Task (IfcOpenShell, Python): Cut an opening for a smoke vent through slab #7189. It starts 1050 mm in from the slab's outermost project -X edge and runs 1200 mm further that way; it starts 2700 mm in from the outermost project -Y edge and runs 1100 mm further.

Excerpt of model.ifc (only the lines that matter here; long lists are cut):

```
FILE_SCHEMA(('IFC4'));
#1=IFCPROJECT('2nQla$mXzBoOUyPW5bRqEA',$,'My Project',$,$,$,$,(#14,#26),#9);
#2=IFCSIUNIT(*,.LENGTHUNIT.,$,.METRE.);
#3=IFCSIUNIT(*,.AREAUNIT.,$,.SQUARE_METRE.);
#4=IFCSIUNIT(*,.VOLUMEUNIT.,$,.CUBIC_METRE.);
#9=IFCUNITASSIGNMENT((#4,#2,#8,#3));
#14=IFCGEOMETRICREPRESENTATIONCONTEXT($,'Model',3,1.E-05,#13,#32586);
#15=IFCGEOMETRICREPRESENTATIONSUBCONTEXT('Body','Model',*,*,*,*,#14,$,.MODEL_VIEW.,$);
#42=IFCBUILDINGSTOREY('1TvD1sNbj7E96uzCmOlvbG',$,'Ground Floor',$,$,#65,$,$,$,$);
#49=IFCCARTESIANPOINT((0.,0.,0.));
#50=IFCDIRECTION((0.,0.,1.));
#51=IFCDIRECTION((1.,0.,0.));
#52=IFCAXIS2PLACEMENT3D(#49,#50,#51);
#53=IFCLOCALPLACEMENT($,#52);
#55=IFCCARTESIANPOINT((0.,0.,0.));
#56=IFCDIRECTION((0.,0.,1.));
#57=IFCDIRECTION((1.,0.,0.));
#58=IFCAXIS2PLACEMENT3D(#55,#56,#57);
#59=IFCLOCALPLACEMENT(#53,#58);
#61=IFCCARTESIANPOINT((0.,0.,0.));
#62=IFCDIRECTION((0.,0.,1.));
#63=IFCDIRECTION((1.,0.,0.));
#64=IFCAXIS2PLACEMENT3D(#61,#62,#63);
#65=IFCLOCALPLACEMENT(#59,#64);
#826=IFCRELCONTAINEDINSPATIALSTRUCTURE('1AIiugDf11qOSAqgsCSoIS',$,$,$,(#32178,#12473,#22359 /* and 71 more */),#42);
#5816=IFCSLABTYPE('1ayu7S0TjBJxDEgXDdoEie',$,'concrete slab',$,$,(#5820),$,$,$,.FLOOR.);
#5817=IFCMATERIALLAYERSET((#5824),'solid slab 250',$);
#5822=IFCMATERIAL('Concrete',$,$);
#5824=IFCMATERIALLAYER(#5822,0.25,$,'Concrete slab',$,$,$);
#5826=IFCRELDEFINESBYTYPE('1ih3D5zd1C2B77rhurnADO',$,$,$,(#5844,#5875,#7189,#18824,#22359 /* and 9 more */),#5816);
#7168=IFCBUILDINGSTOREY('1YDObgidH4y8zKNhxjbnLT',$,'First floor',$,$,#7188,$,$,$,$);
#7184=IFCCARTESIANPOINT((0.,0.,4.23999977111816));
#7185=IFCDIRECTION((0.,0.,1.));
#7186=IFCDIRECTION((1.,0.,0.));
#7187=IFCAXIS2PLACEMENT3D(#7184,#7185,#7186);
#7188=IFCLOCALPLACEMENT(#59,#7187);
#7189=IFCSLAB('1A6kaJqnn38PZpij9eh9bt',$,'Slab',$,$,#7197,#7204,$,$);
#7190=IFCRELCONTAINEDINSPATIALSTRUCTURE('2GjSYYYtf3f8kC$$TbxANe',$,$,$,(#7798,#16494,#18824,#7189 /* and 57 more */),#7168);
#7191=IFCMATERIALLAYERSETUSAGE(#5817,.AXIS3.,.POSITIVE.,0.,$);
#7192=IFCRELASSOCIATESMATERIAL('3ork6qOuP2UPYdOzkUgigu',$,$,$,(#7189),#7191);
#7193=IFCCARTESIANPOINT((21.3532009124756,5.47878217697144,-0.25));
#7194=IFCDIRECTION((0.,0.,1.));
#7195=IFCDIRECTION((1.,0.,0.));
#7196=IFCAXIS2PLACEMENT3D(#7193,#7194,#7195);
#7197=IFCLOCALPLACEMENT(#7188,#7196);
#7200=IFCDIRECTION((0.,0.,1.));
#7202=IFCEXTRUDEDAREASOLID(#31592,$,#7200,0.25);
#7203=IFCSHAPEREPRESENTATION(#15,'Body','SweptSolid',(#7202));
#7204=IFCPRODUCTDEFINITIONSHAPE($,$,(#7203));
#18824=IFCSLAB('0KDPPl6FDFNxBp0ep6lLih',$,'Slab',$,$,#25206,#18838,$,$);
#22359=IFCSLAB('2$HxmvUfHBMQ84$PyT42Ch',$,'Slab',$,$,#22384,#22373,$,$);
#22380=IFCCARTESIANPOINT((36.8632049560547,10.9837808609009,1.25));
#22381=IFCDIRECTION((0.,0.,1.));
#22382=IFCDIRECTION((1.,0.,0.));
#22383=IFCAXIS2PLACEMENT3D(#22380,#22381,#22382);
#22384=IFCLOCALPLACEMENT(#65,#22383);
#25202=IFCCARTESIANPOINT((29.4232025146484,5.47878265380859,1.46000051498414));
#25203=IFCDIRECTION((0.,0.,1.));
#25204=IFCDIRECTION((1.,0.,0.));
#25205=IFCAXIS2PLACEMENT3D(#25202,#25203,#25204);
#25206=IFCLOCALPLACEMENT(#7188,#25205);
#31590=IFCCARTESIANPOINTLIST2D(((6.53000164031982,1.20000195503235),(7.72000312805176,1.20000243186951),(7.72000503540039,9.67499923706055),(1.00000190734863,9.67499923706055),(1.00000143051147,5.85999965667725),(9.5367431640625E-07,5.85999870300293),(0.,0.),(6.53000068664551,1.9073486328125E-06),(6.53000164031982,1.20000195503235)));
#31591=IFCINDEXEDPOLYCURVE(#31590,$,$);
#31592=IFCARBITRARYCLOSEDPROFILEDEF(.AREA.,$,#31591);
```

```python
import numpy as np
import ifcopenshell
import ifcopenshell.api.feature
import ifcopenshell.api.geometry
import ifcopenshell.api.root
import ifcopenshell.geom
import ifcopenshell.util.placement
import ifcopenshell.util.representation
import ifcopenshell.util.shape
import ifcopenshell.util.unit

model = ifcopenshell.open("model.ifc")
unit_scale = ifcopenshell.util.unit.calculate_unit_scale(model)
settings = ifcopenshell.geom.settings()


def volume(element):
    """Net volume in cubic metres, openings subtracted."""
    shape = ifcopenshell.geom.create_shape(settings, element)
    return ifcopenshell.util.shape.get_volume(shape.geometry)


slab = model.by_guid("1A6kaJqnn38PZpij9eh9bt")
before = volume(slab)

# Extent in the slab's own axes, in metres. The edges named are its -X and -Y sides.
slab_shape = ifcopenshell.geom.create_shape(settings, slab)
vertices = ifcopenshell.util.shape.get_vertices(slab_shape.geometry)
x_min, y_min, bottom = vertices.min(axis=0)
top = vertices[:, 2].max()

opening = ifcopenshell.api.root.create_entity(model, ifc_class="IfcOpeningElement", name="Smoke vent opening", predefined_type="OPENING")
context = ifcopenshell.util.representation.get_context(model, "Model", "Body", "MODEL_VIEW")
width, depth = 1.2, 1.1
outline = [(0.0, 0.0), (width, 0.0), (width, depth), (0.0, depth), (0.0, 0.0)]
# Overshoot both faces by 50 mm so the cut is clean.
shape = ifcopenshell.api.geometry.add_slab_representation(
    model, context=context, depth=top - bottom + 0.1, polyline=outline
)
ifcopenshell.api.geometry.assign_representation(model, product=opening, representation=shape)

matrix = ifcopenshell.util.placement.get_local_placement(slab.ObjectPlacement)
matrix[:, 3] = matrix @ np.append(np.array([x_min + 1.05, y_min + 2.7, bottom - 0.05]) / unit_scale, 1.0)
ifcopenshell.api.geometry.edit_object_placement(model, product=opening, matrix=matrix, is_si=False)
ifcopenshell.api.feature.add_feature(model, feature=opening, element=slab)

after = volume(slab)

print(f"slab volume {before:.3f} -> {after:.3f} m3")

model.write("model_v2.ifc")
```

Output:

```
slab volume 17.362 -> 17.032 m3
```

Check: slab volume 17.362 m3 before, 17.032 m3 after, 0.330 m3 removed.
